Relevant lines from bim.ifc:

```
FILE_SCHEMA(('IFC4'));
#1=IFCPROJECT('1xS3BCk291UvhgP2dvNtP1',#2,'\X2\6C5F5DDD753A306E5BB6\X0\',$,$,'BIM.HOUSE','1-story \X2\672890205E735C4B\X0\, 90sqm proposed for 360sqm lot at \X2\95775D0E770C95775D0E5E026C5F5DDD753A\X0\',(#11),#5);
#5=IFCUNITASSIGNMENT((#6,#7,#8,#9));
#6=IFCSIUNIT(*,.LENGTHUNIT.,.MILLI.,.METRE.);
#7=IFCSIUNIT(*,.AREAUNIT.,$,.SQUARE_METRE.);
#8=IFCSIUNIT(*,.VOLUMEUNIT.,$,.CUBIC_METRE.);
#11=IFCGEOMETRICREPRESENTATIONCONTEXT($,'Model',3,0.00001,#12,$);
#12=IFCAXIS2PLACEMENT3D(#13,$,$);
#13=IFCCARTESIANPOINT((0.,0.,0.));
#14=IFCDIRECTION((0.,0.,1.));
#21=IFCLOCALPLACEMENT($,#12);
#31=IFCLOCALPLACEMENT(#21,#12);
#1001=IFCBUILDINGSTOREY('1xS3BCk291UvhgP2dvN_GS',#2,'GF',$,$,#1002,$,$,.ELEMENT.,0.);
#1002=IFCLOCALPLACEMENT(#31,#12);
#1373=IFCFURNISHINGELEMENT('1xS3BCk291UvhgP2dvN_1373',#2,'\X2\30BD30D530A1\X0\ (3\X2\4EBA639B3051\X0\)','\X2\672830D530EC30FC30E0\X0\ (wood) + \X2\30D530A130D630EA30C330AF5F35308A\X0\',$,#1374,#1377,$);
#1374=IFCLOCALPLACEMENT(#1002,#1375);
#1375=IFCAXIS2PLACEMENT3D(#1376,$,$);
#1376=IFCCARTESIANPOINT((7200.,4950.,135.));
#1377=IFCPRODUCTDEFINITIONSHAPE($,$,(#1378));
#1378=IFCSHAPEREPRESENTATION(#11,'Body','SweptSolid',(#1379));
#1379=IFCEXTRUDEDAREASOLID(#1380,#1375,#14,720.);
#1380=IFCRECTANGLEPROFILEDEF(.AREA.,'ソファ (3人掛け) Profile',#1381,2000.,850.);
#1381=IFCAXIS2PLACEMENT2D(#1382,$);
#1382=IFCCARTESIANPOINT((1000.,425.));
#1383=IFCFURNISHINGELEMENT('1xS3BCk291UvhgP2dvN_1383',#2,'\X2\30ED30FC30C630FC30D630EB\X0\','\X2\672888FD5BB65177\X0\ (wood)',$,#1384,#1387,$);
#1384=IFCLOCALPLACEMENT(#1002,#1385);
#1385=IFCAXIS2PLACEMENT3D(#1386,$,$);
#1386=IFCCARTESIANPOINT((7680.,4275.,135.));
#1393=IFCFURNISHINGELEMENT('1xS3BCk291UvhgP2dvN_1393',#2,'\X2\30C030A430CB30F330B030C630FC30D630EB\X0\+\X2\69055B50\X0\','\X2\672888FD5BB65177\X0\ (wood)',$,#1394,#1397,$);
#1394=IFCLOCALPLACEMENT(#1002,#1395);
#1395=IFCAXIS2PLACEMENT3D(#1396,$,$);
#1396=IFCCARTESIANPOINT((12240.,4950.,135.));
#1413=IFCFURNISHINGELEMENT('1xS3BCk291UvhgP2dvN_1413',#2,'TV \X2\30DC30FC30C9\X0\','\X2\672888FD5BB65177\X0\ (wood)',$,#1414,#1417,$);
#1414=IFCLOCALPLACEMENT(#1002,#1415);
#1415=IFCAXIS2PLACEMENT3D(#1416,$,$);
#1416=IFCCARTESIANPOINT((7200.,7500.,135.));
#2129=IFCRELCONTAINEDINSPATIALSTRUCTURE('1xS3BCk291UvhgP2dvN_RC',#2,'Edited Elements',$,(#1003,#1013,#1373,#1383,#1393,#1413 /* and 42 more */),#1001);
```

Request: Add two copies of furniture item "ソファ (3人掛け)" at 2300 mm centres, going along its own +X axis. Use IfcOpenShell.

```python
import ifcopenshell
import ifcopenshell.api.geometry
import ifcopenshell.api.root
import ifcopenshell.util.element
import ifcopenshell.util.placement
import ifcopenshell.util.unit

model = ifcopenshell.open("bim.ifc")
unit_scale = ifcopenshell.util.unit.calculate_unit_scale(model)


def reuse_history(source, copy):
    """copy_class also copies each property set's owner history, people and application; keep the originals."""
    for rel in copy.IsDefinedBy:
        if rel.is_a("IfcRelDefinesByProperties") and (history := rel.RelatingPropertyDefinition.OwnerHistory):
            rel.RelatingPropertyDefinition.OwnerHistory = source.OwnerHistory
            ifcopenshell.util.element.remove_deep2(model, history)


source = model.by_id(1373)
base = ifcopenshell.util.placement.get_local_placement(source.ObjectPlacement)
step = base[:3, 0] * 2.3 / unit_scale

for i in range(1, 3):
    copy = ifcopenshell.api.root.copy_class(model, product=source)
    copy.Representation = ifcopenshell.util.element.copy_deep(
        model, source.Representation, exclude=["IfcGeometricRepresentationContext", "IfcRepresentationMap"]
    )
    reuse_history(source, copy)
    matrix = base.copy()
    matrix[:3, 3] += i * step
    print("added at", matrix[:3, 3].round(3) + 0.0)
    ifcopenshell.api.geometry.edit_object_placement(model, product=copy, matrix=matrix, is_si=False)

model.write("bim_edited.ifc")
```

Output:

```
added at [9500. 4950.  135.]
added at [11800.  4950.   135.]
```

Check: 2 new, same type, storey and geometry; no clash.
